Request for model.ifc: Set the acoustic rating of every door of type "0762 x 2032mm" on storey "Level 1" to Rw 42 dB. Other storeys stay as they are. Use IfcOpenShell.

First a look at what the model holds.

```python
import ifcopenshell
import ifcopenshell.util.element

model = ifcopenshell.open("model.ifc")
print(model.schema)
storey = next(s for s in model.by_type("IfcBuildingStorey") if s.Name == "Level 1")
doors = [e for e in ifcopenshell.util.element.get_decomposition(storey) if e.is_a("IfcDoor")]
seen = {}
for e in doors:
    element_type = ifcopenshell.util.element.get_type(e)
    key = (element_type.Name if element_type != e and element_type else None, ifcopenshell.util.element.get_pset(e, "Pset_DoorCommon", "AcousticRating"))
    seen[key] = seen.get(key, 0) + 1
for (name, value), count in sorted(seen.items(), key=str):
    print(count, "x", name, "|", value)
```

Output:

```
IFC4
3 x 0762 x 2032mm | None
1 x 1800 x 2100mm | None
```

```python
import ifcopenshell
import ifcopenshell.api.pset
import ifcopenshell.util.element

model = ifcopenshell.open("model.ifc")

storey = next(s for s in model.by_type("IfcBuildingStorey") if s.Name == "Level 1")
doors = [e for e in ifcopenshell.util.element.get_decomposition(storey) if e.is_a("IfcDoor")]

count = 0
for e in doors:
    element_type = ifcopenshell.util.element.get_type(e)
    if element_type in (None, e) or element_type.Name != "0762 x 2032mm":
        continue
    # add_pset returns the element's existing set when there is one.
    pset = ifcopenshell.api.pset.add_pset(model, product=e, name="Pset_DoorCommon")
    ifcopenshell.api.pset.edit_pset(model, pset=pset, properties={"AcousticRating": "Rw 42 dB"})
    count += 1

print(count, "doors updated")

model.write("model-out.ifc")
```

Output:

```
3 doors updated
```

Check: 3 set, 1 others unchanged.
